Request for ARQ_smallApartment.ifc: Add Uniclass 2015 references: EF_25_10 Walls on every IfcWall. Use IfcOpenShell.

First a look at what the model holds.

```python
import ifcopenshell

model = ifcopenshell.open("ARQ_smallApartment.ifc")
print(model.schema)
print("classifications:", [c.Name for c in model.by_type("IfcClassification")])
for ifc_class in ("IfcDoor", "IfcRoof", "IfcStair", "IfcWall", "IfcWindow"):
    print(ifc_class, len(model.by_type(ifc_class)))
```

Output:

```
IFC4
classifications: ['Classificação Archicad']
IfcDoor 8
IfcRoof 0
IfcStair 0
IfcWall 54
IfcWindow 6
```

```python
import ifcopenshell
import ifcopenshell.api.classification

model = ifcopenshell.open("ARQ_smallApartment.ifc")

system = ifcopenshell.api.classification.add_classification(model, classification="Uniclass 2015")

codes = {
    "IfcWall": ("EF_25_10", "Walls"),
}
for ifc_class, (code, name) in codes.items():
    products = model.by_type(ifc_class)
    ifcopenshell.api.classification.add_reference(
        model, products=products, classification=system, identification=code, name=name
    )
    print(code, len(products))

model.write("ARQ_smallApartment_v2.ifc")
```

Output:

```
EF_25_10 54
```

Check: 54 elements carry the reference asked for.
